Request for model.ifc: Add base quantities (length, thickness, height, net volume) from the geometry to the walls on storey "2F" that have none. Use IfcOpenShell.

First a look at what the model holds.

```python
import ifcopenshell
import ifcopenshell.util.element
import ifcopenshell.util.unit

model = ifcopenshell.open("model.ifc")
print(model.schema)
for unit_type in ("LENGTHUNIT", "AREAUNIT", "VOLUMEUNIT"):
    print(unit_type, ifcopenshell.util.unit.calculate_unit_scale(model, unit_type))
storey = next(s for s in model.by_type("IfcBuildingStorey") if s.Name == "2F")
walls = [e for e in ifcopenshell.util.element.get_decomposition(storey) if e.is_a("IfcWall")]
for e in sorted(walls, key=lambda e: e.id()):
    print(e.id(), e.is_a(), e.Name, list(ifcopenshell.util.element.get_psets(e, qtos_only=True)), sep=" | ")
```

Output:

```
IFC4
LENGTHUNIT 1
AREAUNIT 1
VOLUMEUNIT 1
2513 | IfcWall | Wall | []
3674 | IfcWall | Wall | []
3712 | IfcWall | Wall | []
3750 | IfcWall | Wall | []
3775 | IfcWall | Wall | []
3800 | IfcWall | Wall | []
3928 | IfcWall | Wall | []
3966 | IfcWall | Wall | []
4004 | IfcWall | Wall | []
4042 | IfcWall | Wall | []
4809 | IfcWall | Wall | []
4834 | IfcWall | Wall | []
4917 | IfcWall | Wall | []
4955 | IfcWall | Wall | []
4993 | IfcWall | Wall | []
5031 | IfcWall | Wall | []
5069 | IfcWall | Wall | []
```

```python
import ifcopenshell
import ifcopenshell.api.pset
import ifcopenshell.geom
import ifcopenshell.util.element
import ifcopenshell.util.shape
import ifcopenshell.util.unit

model = ifcopenshell.open("model.ifc")
unit_scale = ifcopenshell.util.unit.calculate_unit_scale(model)
volume_scale = ifcopenshell.util.unit.calculate_unit_scale(model, "VOLUMEUNIT")
settings = ifcopenshell.geom.settings()

storey = next(s for s in model.by_type("IfcBuildingStorey") if s.Name == "2F")
walls = [e for e in ifcopenshell.util.element.get_decomposition(storey) if e.is_a("IfcWall")]

for e in sorted(walls, key=lambda e: e.id()):
    if ifcopenshell.util.element.get_psets(e, qtos_only=True, should_inherit=False):
        continue
    # Geometry comes back in metres, in the element's own axes.
    shape = ifcopenshell.geom.create_shape(settings, e)
    values = {
        "Length": ifcopenshell.util.shape.get_x(shape.geometry) / unit_scale,
        "Width": ifcopenshell.util.shape.get_y(shape.geometry) / unit_scale,
        "Height": ifcopenshell.util.shape.get_z(shape.geometry) / unit_scale,
        "NetVolume": ifcopenshell.util.shape.get_volume(shape.geometry) / volume_scale,
    }
    qto = ifcopenshell.api.pset.add_qto(model, product=e, name="Qto_WallBaseQuantities")
    ifcopenshell.api.pset.edit_qto(model, qto=qto, properties=values)
    print(e.id(), {k: round(v, 3) for k, v in values.items()})

model.write("model_v2.ifc")
```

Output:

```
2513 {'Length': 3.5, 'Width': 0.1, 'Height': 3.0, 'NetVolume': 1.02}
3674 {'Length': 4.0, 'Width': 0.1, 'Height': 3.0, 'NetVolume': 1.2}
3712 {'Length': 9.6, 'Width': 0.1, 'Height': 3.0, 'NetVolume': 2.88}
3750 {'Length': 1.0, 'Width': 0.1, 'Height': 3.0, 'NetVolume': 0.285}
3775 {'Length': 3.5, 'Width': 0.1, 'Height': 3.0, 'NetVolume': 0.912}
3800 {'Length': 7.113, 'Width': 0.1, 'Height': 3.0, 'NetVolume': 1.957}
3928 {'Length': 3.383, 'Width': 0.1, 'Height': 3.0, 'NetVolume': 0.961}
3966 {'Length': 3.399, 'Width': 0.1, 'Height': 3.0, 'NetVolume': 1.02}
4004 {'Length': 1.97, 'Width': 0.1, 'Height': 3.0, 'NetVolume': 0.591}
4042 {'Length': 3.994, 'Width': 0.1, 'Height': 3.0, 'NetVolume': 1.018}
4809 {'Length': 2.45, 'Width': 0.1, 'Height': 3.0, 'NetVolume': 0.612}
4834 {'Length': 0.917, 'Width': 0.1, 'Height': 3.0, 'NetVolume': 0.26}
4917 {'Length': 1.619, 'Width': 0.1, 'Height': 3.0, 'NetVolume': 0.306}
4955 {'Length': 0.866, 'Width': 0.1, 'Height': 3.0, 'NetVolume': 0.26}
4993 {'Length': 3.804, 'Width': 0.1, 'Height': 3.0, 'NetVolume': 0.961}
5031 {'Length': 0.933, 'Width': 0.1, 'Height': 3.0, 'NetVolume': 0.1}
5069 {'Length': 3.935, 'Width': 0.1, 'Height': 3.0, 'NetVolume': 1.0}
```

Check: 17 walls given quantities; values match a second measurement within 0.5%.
